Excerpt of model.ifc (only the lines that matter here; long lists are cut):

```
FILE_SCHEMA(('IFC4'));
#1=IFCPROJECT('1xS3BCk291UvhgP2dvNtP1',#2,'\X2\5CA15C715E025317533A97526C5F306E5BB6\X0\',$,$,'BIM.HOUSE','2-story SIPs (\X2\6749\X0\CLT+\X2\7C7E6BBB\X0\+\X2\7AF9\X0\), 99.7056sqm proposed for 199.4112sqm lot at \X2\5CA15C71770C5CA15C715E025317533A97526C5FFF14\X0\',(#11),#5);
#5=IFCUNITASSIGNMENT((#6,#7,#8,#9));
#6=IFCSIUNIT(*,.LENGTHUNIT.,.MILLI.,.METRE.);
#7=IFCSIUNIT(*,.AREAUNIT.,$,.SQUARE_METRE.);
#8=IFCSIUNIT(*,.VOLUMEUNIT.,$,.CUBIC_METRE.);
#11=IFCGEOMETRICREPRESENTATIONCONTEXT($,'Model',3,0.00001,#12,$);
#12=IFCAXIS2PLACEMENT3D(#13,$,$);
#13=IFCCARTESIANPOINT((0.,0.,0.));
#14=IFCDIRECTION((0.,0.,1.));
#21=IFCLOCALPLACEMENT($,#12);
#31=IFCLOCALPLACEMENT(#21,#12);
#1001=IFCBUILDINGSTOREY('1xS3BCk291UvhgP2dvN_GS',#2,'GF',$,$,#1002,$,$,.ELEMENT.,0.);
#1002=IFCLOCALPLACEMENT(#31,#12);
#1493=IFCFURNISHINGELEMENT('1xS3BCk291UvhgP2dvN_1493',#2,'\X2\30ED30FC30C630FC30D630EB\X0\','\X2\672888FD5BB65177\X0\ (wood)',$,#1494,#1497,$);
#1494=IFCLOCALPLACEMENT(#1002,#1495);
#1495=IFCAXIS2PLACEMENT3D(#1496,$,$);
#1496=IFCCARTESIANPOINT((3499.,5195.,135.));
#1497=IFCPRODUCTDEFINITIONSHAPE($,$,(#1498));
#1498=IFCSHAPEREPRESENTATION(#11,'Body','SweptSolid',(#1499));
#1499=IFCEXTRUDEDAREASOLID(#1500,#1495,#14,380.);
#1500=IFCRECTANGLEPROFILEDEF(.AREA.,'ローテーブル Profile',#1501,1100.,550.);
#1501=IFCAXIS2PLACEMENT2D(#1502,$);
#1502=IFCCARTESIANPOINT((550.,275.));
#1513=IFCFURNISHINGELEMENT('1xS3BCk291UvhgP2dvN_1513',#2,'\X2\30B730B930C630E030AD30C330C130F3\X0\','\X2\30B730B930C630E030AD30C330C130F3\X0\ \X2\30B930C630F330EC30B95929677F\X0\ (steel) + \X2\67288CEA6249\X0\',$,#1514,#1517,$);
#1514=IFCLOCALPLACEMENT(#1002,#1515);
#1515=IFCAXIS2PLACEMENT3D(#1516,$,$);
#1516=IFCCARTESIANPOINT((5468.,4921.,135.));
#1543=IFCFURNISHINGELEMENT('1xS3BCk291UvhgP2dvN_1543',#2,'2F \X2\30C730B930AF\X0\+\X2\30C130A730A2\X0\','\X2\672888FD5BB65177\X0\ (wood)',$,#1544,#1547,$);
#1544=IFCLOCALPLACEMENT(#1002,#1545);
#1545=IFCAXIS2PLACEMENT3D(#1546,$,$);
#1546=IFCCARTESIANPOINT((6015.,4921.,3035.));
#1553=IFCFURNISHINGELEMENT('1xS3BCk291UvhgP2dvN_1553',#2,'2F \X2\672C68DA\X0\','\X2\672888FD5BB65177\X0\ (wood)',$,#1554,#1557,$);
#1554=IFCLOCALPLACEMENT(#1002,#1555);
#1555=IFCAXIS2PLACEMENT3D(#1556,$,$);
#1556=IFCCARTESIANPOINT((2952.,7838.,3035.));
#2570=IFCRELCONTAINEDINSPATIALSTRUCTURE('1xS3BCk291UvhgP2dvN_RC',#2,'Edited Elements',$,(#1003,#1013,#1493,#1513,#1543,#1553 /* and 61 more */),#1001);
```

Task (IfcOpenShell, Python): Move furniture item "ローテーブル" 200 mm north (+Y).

```python
import ifcopenshell
import ifcopenshell.api.geometry
import ifcopenshell.util.placement
import ifcopenshell.util.unit

model = ifcopenshell.open("model.ifc")
unit_scale = ifcopenshell.util.unit.calculate_unit_scale(model)

item = model.by_guid("1xS3BCk291UvhgP2dvN_1493")
matrix = ifcopenshell.util.placement.get_local_placement(item.ObjectPlacement)
matrix[1, 3] += 0.2 / unit_scale
ifcopenshell.api.geometry.edit_object_placement(model, product=item, matrix=matrix, is_si=False)

print(ifcopenshell.util.placement.get_local_placement(item.ObjectPlacement).round(3) + 0.0)

model.write("model_edited.ifc")
```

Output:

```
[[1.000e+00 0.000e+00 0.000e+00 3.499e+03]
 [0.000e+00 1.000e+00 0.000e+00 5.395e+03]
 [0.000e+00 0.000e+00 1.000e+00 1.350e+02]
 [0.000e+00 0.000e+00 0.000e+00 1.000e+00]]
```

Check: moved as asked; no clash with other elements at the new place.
